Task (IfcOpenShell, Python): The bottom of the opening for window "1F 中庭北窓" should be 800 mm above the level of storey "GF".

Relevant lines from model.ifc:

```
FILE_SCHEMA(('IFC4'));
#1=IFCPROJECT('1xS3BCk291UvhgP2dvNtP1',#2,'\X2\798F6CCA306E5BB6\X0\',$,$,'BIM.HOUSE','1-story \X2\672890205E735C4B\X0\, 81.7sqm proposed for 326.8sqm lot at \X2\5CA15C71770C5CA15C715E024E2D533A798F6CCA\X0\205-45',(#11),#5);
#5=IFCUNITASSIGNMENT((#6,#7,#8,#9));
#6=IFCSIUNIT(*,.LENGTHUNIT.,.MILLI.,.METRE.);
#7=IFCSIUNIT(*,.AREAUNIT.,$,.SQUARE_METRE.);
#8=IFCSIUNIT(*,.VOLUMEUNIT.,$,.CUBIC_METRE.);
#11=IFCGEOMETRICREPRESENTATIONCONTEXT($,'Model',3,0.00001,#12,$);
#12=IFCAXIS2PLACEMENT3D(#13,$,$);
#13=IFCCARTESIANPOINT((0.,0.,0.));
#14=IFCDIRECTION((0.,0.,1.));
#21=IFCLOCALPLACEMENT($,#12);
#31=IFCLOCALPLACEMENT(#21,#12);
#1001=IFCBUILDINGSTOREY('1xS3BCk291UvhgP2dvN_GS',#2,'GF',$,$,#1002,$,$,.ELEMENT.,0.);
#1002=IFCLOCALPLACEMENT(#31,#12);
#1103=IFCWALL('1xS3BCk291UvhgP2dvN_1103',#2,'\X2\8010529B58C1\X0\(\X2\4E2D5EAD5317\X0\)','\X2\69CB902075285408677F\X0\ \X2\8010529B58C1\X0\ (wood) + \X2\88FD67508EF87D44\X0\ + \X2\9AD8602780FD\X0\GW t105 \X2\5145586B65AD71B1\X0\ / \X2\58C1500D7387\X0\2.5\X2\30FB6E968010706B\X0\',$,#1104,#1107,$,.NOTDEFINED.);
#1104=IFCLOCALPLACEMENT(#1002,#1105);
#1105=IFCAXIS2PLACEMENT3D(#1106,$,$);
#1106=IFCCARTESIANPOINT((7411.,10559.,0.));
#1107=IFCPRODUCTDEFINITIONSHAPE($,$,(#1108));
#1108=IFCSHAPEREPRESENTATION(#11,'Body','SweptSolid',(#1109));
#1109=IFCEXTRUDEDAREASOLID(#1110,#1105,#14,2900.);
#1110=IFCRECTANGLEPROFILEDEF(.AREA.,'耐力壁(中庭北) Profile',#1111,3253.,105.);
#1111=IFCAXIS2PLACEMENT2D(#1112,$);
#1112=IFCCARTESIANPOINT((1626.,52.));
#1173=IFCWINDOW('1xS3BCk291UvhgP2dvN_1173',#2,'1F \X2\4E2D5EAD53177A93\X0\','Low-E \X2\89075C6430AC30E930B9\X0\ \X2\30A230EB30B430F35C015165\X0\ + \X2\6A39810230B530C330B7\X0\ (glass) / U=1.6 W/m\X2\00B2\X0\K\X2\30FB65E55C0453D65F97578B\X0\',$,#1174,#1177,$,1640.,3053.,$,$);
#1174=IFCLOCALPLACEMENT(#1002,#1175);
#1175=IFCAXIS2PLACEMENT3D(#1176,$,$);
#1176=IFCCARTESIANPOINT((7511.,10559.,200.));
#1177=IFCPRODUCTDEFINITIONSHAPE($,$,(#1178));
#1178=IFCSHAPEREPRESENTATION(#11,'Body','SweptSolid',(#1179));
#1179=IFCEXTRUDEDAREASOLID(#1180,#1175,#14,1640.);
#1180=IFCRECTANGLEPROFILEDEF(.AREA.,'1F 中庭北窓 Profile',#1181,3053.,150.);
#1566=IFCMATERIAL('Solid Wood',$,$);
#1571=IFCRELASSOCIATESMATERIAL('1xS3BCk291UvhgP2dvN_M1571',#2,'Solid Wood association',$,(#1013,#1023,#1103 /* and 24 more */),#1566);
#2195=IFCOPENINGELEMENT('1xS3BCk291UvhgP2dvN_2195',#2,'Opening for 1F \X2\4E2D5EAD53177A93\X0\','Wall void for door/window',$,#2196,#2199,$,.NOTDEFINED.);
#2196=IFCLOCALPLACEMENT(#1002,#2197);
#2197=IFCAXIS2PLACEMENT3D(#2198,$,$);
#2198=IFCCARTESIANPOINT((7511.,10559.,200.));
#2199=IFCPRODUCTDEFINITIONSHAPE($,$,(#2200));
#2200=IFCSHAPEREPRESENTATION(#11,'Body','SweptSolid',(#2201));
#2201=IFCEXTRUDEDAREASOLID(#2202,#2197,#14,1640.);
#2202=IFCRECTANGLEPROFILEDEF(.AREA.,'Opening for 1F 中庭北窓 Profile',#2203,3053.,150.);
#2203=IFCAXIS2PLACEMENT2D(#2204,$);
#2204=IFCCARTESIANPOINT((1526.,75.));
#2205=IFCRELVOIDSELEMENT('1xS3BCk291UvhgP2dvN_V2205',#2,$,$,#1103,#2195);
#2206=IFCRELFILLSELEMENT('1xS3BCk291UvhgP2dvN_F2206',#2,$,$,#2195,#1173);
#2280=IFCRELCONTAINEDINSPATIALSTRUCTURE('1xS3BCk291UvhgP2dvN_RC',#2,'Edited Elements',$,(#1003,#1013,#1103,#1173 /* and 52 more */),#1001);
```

```python
import numpy as np
import ifcopenshell
import ifcopenshell.api.geometry
import ifcopenshell.geom
import ifcopenshell.util.element
import ifcopenshell.util.placement
import ifcopenshell.util.shape
import ifcopenshell.util.unit

model = ifcopenshell.open("model.ifc")
unit_scale = ifcopenshell.util.unit.calculate_unit_scale(model)

window = model.by_guid("1xS3BCk291UvhgP2dvN_1173")
opening = window.FillsVoids[0].RelatingOpeningElement
storey = ifcopenshell.util.element.get_container(window, ifc_class="IfcBuildingStorey")
level = ifcopenshell.util.placement.get_local_placement(storey.ObjectPlacement)[2, 3]

# The opening's origin need not be at the sill, so measure its lowest point.
shape = ifcopenshell.geom.create_shape(ifcopenshell.geom.settings(), opening)
bottom = ifcopenshell.util.shape.get_shape_bottom_elevation(shape, shape.geometry) / unit_scale
dz = level + 0.8 / unit_scale - bottom

shift = np.array([0.0, 0.0, dz])
# The window is not placed relative to its opening, so move both.
for product in (opening, window):
    matrix = ifcopenshell.util.placement.get_local_placement(product.ObjectPlacement)
    matrix[:3, 3] += shift
    ifcopenshell.api.geometry.edit_object_placement(model, product=product, matrix=matrix, is_si=False)

print(f"moved by {dz * unit_scale:+.3f} m")

model.write("model_v2.ifc")
```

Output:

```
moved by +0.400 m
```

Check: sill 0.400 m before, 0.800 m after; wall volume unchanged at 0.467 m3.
